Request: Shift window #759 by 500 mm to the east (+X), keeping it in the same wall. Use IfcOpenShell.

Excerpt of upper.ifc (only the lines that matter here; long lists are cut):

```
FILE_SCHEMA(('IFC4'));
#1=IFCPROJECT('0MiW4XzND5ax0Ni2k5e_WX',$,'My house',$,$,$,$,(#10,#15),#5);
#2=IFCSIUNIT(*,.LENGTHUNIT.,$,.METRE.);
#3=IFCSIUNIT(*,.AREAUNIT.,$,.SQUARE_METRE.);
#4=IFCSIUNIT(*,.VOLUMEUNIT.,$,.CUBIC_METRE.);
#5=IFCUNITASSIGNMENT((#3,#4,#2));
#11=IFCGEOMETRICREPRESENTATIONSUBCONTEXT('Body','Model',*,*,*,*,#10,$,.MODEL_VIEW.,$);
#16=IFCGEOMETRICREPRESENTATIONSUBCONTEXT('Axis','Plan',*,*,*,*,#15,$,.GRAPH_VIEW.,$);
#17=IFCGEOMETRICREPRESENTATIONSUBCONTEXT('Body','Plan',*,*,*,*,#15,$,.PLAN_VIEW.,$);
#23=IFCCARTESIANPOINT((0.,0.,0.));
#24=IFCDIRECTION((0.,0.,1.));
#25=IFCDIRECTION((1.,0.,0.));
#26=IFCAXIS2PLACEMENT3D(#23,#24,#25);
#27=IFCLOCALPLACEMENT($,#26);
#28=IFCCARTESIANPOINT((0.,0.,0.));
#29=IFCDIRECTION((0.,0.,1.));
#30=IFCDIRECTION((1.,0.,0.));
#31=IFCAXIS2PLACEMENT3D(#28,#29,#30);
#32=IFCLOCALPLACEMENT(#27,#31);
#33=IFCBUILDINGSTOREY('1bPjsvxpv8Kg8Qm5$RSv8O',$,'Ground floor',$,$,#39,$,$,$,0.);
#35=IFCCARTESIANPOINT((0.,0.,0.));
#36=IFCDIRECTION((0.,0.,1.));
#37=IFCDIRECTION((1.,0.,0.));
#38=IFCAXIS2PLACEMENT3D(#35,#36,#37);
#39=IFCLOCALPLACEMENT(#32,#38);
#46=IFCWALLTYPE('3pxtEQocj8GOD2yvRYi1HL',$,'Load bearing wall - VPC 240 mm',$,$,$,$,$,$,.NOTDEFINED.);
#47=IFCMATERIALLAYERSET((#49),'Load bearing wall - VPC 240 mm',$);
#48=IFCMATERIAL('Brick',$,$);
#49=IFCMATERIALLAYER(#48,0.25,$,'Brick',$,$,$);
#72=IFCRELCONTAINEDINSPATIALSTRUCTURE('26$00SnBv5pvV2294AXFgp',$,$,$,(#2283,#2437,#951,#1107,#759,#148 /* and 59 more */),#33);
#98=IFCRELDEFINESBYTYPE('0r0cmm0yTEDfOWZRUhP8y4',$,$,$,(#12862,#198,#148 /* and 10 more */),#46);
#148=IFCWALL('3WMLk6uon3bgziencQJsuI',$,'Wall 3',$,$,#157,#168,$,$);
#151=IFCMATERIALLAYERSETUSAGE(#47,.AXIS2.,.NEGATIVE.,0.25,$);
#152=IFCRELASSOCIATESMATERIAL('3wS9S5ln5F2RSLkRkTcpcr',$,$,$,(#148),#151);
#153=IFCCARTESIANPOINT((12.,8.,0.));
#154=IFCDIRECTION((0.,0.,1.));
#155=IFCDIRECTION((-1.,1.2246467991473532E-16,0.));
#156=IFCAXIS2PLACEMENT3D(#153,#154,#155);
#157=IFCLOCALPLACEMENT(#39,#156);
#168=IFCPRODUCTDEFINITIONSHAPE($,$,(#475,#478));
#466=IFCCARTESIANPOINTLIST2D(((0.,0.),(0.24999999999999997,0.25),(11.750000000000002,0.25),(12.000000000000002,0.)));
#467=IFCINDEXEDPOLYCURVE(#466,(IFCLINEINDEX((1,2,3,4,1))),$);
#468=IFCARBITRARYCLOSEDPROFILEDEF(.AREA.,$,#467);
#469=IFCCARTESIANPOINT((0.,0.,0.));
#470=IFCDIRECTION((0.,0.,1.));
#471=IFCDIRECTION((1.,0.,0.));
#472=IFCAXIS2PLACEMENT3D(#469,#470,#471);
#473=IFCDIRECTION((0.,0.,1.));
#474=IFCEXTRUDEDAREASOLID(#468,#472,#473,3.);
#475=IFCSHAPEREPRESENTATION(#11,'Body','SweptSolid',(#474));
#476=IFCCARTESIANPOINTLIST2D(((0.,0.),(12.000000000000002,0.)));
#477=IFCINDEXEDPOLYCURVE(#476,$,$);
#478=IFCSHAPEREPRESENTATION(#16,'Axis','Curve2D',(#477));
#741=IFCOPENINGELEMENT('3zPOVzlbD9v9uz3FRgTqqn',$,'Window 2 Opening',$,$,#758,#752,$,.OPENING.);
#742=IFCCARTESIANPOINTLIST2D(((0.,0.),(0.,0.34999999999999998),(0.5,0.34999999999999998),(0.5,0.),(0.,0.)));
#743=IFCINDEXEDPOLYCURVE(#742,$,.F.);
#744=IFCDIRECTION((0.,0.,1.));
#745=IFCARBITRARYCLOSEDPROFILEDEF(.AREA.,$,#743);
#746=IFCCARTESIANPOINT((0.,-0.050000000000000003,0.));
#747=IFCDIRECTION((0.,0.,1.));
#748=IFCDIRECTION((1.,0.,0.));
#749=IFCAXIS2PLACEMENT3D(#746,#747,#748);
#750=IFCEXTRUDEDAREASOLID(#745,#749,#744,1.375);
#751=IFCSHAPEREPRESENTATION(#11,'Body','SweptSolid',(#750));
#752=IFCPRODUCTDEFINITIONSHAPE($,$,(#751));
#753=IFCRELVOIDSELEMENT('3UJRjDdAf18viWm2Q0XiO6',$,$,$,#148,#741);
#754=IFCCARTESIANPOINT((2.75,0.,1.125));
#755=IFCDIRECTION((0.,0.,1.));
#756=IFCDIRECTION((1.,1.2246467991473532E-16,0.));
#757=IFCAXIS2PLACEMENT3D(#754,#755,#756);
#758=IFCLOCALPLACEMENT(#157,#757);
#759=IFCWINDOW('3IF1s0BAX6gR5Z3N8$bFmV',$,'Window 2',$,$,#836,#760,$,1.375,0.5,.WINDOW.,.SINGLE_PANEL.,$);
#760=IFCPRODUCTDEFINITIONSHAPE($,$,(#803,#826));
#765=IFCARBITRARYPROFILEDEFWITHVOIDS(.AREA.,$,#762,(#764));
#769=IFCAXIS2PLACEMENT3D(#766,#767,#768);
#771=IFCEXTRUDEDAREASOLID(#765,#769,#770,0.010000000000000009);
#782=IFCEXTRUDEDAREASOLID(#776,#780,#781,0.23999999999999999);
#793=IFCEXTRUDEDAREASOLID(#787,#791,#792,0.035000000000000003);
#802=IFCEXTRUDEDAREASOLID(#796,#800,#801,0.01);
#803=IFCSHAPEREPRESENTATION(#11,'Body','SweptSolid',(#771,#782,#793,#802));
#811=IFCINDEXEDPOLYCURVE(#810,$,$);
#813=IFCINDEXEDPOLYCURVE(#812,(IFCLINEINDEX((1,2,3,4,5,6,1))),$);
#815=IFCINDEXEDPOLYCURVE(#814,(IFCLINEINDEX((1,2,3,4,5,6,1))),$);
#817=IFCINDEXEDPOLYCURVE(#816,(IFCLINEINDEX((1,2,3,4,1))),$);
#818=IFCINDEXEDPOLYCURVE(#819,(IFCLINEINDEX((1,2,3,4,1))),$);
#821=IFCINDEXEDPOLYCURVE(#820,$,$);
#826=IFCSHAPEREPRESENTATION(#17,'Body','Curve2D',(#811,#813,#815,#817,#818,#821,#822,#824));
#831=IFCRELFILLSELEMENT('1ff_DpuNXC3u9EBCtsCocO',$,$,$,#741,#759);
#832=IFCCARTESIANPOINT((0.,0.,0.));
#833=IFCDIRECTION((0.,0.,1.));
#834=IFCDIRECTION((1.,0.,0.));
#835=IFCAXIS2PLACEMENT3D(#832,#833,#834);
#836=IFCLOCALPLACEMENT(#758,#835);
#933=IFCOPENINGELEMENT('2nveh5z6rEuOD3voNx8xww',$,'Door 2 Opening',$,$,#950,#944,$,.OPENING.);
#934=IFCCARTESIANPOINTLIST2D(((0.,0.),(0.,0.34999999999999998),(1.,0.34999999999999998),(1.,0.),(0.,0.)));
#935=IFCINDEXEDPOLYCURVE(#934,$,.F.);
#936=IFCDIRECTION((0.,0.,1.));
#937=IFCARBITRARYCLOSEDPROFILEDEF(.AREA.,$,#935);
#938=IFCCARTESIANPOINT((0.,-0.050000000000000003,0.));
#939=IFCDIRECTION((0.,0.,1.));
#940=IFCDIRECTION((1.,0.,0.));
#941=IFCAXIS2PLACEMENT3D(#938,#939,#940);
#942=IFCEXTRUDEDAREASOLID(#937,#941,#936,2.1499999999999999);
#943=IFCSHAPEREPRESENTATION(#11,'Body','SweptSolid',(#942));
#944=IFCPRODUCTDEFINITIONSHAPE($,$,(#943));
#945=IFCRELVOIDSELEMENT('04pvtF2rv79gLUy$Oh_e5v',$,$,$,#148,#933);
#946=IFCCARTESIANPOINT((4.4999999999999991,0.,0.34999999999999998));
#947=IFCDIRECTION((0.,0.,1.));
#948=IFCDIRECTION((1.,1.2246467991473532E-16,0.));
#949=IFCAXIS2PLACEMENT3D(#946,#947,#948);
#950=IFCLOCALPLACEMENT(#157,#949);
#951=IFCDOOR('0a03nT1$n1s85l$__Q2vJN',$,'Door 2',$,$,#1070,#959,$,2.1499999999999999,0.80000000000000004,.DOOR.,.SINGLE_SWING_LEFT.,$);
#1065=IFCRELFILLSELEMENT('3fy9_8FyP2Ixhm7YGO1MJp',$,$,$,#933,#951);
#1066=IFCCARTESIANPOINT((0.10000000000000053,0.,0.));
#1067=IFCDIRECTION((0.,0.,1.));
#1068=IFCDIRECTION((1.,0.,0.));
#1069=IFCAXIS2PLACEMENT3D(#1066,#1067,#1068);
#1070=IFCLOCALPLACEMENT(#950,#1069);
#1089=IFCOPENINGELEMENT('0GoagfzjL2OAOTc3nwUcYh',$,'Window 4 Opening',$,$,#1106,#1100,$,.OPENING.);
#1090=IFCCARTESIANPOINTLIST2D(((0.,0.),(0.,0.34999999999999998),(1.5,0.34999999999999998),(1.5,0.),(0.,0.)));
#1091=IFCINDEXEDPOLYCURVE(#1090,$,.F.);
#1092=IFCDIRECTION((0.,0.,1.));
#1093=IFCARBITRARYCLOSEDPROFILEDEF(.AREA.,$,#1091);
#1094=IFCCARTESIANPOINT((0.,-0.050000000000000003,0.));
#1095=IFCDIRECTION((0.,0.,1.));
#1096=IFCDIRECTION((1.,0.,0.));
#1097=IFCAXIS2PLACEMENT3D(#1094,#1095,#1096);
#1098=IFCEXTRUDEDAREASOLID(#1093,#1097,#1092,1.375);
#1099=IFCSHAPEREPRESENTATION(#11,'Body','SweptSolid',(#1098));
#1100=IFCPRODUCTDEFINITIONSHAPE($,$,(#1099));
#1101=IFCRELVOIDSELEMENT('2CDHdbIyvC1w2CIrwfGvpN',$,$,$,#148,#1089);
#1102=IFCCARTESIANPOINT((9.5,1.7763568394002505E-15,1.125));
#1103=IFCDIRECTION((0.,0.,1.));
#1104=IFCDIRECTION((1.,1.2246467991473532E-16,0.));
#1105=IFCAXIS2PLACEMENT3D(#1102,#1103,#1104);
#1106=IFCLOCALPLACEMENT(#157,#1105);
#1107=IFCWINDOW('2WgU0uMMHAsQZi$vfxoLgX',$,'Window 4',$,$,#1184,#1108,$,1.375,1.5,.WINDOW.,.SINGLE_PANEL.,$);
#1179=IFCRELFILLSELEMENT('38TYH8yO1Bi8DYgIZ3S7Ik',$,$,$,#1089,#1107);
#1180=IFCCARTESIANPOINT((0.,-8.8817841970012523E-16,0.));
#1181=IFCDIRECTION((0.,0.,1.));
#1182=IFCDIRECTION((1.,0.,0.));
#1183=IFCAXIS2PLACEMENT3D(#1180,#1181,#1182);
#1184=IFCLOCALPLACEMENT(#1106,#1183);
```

```python
import ifcopenshell
import ifcopenshell.api.geometry
import ifcopenshell.util.placement
import ifcopenshell.util.unit

model = ifcopenshell.open("upper.ifc")
unit_scale = ifcopenshell.util.unit.calculate_unit_scale(model)

window = model.by_id(759)
opening = window.FillsVoids[0].RelatingOpeningElement
wall = opening.VoidsElements[0].RelatingBuildingElement

wall_matrix = ifcopenshell.util.placement.get_local_placement(wall.ObjectPlacement)
shift = wall_matrix[:3, 0] * -0.5 / unit_scale
before = ifcopenshell.util.placement.get_local_placement(window.ObjectPlacement)[:3, 3].copy()

# The window is placed relative to its opening, so it follows when the opening moves.
matrix = ifcopenshell.util.placement.get_local_placement(opening.ObjectPlacement)
matrix[:3, 3] += shift
ifcopenshell.api.geometry.edit_object_placement(
    model, product=opening, matrix=matrix, is_si=False, should_transform_children=True
)

after = ifcopenshell.util.placement.get_local_placement(window.ObjectPlacement)[:3, 3]
print("window moved by", (after - before).round(3) + 0.0)

model.write("upper_updated.ifc")
```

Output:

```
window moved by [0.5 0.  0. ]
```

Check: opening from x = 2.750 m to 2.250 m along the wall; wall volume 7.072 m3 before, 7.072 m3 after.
